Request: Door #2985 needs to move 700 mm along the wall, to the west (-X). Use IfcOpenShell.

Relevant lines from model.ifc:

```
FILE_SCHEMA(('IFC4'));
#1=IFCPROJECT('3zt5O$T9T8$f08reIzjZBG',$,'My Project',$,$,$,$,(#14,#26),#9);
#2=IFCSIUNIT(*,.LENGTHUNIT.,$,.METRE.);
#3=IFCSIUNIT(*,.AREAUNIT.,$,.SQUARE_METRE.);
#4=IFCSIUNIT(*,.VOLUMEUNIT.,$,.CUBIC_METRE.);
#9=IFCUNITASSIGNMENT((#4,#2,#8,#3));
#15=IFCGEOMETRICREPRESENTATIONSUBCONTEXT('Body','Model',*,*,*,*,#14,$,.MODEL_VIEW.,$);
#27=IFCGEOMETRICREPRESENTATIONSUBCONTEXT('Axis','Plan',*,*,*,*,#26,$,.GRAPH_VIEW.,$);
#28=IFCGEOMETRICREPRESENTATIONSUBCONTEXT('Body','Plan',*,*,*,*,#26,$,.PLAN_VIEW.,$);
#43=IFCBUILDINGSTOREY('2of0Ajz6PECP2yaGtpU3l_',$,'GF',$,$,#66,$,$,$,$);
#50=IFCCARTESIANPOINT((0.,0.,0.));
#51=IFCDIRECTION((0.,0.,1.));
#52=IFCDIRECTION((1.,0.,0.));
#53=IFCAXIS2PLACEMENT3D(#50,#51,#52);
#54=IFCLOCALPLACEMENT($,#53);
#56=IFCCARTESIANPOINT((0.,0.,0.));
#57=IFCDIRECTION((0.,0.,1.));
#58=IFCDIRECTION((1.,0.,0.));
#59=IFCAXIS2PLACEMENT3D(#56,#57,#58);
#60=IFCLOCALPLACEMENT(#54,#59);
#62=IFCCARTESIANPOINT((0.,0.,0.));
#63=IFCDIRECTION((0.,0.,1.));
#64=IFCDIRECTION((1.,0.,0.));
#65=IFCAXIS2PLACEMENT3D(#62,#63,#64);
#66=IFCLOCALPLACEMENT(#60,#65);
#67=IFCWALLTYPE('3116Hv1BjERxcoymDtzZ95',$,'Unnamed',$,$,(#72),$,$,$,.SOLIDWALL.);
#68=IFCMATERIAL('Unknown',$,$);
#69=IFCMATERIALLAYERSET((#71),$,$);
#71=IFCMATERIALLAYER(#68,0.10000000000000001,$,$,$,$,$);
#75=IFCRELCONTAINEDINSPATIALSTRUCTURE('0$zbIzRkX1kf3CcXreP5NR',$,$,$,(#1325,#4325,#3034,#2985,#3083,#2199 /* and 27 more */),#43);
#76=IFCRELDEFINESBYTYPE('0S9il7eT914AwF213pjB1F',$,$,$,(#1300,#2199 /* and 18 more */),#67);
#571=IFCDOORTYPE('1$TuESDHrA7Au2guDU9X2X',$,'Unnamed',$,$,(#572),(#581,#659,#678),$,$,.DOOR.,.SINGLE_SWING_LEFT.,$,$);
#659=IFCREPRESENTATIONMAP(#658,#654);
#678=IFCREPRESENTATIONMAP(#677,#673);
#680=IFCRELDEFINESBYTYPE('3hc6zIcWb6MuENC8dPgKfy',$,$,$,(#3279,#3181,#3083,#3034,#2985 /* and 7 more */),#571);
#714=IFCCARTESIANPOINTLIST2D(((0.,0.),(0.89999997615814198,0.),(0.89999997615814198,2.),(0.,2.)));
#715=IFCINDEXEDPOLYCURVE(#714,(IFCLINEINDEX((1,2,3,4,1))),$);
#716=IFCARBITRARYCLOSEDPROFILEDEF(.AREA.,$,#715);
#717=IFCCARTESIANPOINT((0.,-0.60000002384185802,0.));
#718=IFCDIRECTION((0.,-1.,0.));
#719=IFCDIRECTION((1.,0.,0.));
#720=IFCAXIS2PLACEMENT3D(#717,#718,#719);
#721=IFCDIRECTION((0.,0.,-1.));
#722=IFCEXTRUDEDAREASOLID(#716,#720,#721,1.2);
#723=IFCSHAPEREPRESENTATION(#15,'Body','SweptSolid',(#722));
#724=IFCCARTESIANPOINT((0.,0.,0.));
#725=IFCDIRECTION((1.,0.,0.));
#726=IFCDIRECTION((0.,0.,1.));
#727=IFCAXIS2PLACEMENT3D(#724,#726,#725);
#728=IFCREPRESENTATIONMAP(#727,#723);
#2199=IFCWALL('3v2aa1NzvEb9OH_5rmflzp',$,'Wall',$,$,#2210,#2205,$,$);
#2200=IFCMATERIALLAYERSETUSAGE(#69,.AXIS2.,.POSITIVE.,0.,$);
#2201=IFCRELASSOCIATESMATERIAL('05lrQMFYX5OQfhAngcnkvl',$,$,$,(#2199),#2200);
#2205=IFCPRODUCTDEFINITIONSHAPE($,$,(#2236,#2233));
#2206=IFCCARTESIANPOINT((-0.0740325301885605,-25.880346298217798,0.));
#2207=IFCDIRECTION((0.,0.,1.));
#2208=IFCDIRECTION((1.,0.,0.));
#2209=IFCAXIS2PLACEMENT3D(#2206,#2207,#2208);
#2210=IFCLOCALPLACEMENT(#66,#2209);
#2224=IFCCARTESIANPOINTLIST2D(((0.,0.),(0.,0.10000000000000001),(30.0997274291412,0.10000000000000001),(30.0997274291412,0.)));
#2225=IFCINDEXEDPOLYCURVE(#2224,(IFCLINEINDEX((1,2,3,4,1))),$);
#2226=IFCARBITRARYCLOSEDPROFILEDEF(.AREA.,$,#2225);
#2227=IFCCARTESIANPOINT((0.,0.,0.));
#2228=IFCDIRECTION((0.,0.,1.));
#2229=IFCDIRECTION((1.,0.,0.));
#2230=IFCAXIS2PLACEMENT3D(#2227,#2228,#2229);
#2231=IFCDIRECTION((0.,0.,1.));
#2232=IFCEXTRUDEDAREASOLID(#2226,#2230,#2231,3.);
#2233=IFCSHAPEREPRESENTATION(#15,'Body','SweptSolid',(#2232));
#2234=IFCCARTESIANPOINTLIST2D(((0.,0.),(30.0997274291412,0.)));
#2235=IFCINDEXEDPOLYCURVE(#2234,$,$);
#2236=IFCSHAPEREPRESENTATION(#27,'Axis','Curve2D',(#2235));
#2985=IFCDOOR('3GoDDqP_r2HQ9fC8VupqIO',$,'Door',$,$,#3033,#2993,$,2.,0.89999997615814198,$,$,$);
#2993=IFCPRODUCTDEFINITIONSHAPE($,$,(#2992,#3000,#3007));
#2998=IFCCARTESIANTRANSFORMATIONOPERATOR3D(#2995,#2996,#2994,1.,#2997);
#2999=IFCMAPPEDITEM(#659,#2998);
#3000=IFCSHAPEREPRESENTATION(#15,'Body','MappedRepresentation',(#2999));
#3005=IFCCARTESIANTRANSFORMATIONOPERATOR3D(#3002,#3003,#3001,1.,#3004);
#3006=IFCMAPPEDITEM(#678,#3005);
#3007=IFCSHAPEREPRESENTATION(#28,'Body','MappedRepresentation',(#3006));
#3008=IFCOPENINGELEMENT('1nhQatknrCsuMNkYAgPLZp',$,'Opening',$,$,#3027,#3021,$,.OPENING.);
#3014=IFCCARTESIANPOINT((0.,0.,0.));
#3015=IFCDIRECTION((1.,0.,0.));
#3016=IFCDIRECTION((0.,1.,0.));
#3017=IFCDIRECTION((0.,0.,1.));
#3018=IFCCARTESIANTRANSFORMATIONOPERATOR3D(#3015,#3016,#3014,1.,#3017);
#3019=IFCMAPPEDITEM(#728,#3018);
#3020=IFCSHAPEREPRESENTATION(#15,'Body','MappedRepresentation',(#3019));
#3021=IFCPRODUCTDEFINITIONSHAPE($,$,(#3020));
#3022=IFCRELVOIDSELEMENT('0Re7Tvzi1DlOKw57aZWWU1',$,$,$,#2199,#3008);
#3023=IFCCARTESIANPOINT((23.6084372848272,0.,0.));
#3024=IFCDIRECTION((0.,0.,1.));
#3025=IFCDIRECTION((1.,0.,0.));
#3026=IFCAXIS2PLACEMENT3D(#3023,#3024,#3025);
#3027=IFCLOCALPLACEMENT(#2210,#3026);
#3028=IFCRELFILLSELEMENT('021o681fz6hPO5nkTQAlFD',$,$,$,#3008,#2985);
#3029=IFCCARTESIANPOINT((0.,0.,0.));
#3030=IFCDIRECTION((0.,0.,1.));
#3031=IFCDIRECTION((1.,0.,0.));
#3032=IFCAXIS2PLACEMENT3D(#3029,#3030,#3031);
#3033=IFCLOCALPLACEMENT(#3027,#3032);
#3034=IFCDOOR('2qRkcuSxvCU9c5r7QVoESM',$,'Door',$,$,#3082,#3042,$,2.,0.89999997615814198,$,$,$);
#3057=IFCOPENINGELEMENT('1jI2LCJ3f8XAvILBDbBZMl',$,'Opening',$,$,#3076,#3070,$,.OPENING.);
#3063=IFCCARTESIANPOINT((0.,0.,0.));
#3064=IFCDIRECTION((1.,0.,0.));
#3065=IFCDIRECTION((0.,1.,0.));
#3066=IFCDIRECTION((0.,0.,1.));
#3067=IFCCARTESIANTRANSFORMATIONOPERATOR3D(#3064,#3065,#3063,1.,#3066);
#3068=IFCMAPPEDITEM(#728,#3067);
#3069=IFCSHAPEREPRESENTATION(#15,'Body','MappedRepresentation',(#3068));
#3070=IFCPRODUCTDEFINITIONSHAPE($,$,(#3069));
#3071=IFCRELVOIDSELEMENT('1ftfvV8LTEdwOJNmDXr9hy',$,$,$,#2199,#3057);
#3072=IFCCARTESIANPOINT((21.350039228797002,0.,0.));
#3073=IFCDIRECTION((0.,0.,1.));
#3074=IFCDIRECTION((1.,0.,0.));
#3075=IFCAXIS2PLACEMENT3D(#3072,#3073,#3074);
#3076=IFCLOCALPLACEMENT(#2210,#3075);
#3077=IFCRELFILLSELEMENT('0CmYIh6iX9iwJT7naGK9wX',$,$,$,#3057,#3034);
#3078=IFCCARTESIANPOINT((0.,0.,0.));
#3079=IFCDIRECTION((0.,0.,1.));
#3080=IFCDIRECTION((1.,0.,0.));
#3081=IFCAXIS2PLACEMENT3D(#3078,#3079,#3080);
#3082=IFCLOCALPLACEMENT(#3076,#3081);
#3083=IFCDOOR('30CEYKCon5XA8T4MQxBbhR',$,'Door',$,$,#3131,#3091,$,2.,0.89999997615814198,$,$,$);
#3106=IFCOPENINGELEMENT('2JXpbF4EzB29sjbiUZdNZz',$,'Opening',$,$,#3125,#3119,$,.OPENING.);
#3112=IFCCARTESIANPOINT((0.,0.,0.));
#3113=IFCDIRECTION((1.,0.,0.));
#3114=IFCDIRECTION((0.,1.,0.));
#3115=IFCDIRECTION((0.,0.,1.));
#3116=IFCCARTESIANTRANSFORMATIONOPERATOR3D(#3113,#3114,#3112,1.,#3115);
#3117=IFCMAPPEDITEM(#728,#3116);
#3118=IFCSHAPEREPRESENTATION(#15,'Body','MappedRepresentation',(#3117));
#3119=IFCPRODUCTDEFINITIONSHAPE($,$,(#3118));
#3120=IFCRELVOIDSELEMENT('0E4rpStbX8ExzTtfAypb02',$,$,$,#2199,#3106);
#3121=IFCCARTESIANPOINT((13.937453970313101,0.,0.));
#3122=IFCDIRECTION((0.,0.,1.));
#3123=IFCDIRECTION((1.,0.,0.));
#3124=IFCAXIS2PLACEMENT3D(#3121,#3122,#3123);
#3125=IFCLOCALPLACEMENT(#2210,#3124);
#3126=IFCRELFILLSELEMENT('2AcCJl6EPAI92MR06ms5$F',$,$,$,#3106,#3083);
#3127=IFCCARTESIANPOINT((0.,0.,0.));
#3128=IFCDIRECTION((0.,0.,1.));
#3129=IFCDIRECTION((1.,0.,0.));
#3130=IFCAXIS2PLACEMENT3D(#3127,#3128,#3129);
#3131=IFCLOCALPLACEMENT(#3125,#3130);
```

```python
import ifcopenshell
import ifcopenshell.api.geometry
import ifcopenshell.util.placement
import ifcopenshell.util.unit

model = ifcopenshell.open("model.ifc")
unit_scale = ifcopenshell.util.unit.calculate_unit_scale(model)

door = model.by_guid("3GoDDqP_r2HQ9fC8VupqIO")
opening = door.FillsVoids[0].RelatingOpeningElement
wall = opening.VoidsElements[0].RelatingBuildingElement

wall_matrix = ifcopenshell.util.placement.get_local_placement(wall.ObjectPlacement)
shift = wall_matrix[:3, 0] * -0.7 / unit_scale
before = ifcopenshell.util.placement.get_local_placement(door.ObjectPlacement)[:3, 3].copy()

# The door is placed relative to its opening, so it follows when the opening moves.
matrix = ifcopenshell.util.placement.get_local_placement(opening.ObjectPlacement)
matrix[:3, 3] += shift
ifcopenshell.api.geometry.edit_object_placement(
    model, product=opening, matrix=matrix, is_si=False, should_transform_children=True
)

after = ifcopenshell.util.placement.get_local_placement(door.ObjectPlacement)[:3, 3]
print("door moved by", (after - before).round(3) + 0.0)

model.write("model_edited.ifc")
```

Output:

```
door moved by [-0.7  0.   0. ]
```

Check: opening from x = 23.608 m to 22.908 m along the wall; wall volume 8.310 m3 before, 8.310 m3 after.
